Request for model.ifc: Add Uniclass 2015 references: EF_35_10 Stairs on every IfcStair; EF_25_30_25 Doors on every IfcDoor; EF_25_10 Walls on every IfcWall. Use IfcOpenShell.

First a look at what the model holds.

```python
import ifcopenshell

model = ifcopenshell.open("model.ifc")
print(model.schema)
print("classifications:", [c.Name for c in model.by_type("IfcClassification")])
for ifc_class in ("IfcDoor", "IfcRoof", "IfcStair", "IfcWall", "IfcWindow"):
    print(ifc_class, len(model.by_type(ifc_class)))
```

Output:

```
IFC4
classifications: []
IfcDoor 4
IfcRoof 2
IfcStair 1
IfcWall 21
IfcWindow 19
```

```python
import ifcopenshell
import ifcopenshell.api.classification

model = ifcopenshell.open("model.ifc")

system = ifcopenshell.api.classification.add_classification(model, classification="Uniclass 2015")

codes = {
    "IfcStair": ("EF_35_10", "Stairs"),
    "IfcDoor": ("EF_25_30_25", "Doors"),
    "IfcWall": ("EF_25_10", "Walls"),
}
for ifc_class, (code, name) in codes.items():
    products = model.by_type(ifc_class)
    ifcopenshell.api.classification.add_reference(
        model, products=products, classification=system, identification=code, name=name
    )
    print(code, len(products))

model.write("model_updated.ifc")
```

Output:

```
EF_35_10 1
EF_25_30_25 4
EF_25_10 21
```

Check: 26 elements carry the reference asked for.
